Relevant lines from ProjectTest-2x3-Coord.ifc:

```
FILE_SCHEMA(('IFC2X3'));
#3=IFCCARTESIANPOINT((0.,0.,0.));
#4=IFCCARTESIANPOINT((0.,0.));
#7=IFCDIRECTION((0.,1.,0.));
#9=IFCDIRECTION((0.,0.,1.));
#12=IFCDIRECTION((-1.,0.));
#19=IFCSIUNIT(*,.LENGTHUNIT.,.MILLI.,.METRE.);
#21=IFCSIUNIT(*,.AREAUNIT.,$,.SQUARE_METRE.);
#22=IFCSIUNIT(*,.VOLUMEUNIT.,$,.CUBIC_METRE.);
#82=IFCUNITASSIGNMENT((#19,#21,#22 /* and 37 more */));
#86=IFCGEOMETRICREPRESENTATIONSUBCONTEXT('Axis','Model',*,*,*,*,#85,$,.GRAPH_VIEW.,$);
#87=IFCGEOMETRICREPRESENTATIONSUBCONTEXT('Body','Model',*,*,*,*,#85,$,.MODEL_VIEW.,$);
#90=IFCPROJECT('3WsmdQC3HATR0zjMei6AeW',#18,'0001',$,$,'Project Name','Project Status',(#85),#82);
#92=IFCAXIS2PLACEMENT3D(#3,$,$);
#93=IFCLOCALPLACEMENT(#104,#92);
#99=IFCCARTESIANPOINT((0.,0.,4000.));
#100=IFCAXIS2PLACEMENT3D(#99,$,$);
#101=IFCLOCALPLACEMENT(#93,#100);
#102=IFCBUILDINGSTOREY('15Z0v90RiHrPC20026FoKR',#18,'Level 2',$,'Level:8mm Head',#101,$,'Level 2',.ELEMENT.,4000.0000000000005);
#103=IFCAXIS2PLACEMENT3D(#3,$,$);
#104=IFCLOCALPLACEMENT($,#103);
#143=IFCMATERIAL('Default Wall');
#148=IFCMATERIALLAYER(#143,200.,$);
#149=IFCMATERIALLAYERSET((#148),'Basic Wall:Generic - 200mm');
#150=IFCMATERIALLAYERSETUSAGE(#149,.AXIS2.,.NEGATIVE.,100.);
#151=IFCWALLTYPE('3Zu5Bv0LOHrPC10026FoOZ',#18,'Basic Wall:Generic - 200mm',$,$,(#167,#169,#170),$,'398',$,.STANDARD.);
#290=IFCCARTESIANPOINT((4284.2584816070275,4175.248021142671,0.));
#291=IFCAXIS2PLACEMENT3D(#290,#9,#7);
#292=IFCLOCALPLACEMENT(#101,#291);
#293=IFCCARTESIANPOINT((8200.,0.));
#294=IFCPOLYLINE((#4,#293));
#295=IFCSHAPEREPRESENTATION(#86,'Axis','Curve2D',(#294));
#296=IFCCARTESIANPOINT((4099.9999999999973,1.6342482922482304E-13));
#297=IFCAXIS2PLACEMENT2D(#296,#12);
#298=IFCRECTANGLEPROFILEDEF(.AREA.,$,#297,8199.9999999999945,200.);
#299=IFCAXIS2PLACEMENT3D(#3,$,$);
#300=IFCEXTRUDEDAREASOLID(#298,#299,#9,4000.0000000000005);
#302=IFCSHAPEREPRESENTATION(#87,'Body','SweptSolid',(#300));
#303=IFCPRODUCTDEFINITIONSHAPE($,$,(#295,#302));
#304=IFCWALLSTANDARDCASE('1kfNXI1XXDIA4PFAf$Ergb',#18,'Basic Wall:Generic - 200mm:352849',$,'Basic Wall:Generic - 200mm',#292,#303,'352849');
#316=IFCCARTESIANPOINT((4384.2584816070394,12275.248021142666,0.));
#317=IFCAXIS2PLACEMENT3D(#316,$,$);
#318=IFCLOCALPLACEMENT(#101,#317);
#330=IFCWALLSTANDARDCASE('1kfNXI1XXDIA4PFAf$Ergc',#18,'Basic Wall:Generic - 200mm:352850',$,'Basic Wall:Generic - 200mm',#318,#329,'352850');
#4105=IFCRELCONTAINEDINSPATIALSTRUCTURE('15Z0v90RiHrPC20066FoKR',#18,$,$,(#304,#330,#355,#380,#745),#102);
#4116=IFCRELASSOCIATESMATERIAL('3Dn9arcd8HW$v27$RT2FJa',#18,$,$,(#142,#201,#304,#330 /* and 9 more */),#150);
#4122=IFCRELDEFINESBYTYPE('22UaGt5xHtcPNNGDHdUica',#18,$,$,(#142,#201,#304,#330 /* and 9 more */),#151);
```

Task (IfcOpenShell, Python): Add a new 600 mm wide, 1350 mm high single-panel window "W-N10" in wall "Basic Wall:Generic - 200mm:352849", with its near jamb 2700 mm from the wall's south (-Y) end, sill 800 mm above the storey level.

```python
import numpy as np
import ifcopenshell
import ifcopenshell.api.feature
import ifcopenshell.api.geometry
import ifcopenshell.api.root
import ifcopenshell.api.spatial
import ifcopenshell.api.type
import ifcopenshell.geom
import ifcopenshell.util.element
import ifcopenshell.util.placement
import ifcopenshell.util.representation
import ifcopenshell.util.shape
import ifcopenshell.util.unit

model = ifcopenshell.open("ProjectTest-2x3-Coord.ifc")
unit_scale = ifcopenshell.util.unit.calculate_unit_scale(model)
settings = ifcopenshell.geom.settings()


def volume(element):
    """Net volume in cubic metres, openings subtracted."""
    shape = ifcopenshell.geom.create_shape(settings, element)
    return ifcopenshell.util.shape.get_volume(shape.geometry)


wall = model.by_guid("1kfNXI1XXDIA4PFAf$Ergb")
storey = ifcopenshell.util.element.get_container(wall, ifc_class="IfcBuildingStorey")
context = ifcopenshell.util.representation.get_context(model, "Model", "Body", "MODEL_VIEW")
before = volume(wall)

width, height, from_end, sill = 0.6, 1.35, 2.7, 0.8  # metres

# The wall runs along its own X axis, and the end named is its -X end.
wall_shape = ifcopenshell.geom.create_shape(settings, wall)
x, y, z = ifcopenshell.util.shape.get_vertices(wall_shape.geometry).T
start = x.min() + from_end
face, thickness = float(y.min()), float(y.max() - y.min())
wall_matrix = ifcopenshell.util.placement.get_local_placement(wall.ObjectPlacement)
level = ifcopenshell.util.placement.get_local_placement(storey.ObjectPlacement)[2, 3]


def in_wall(x, y):
    """Placement at x, y metres in the wall's axes, at sill height."""
    matrix = wall_matrix.copy()
    matrix[:, 3] = wall_matrix @ np.array([x / unit_scale, y / unit_scale, 0.0, 1.0])
    matrix[2, 3] = level + sill / unit_scale
    return matrix


# Opening: a box that overshoots both wall faces by 50 mm.
opening = ifcopenshell.api.root.create_entity(model, ifc_class="IfcOpeningElement")
box = ifcopenshell.api.geometry.add_wall_representation(
    model, context=context, length=width, height=height, thickness=thickness + 0.1
)
ifcopenshell.api.geometry.assign_representation(model, product=opening, representation=box)
ifcopenshell.api.geometry.edit_object_placement(model, product=opening, matrix=in_wall(start, face - 0.05), is_si=False)
ifcopenshell.api.feature.add_feature(model, feature=opening, element=wall)

window = ifcopenshell.api.root.create_entity(model, ifc_class="IfcWindow", name="W-N10")
window.OverallWidth, window.OverallHeight = width / unit_scale, height / unit_scale
body = ifcopenshell.api.geometry.add_window_representation(
    model,
    context=context,
    overall_width=window.OverallWidth,
    overall_height=window.OverallHeight,
    partition_type="SINGLE_PANEL",
)
ifcopenshell.api.geometry.assign_representation(model, product=window, representation=body)
ifcopenshell.api.spatial.assign_container(model, products=[window], relating_structure=storey)
fills = ifcopenshell.api.feature.add_filling(model, opening=opening, element=window)
fills.OwnerHistory = window.OwnerHistory  # required in IFC2X3

# IFC2X3 keeps the operation on the window style.
style = ifcopenshell.api.root.create_entity(model, ifc_class="IfcWindowStyle", name="W-N10")
style.OperationType, style.ConstructionType = "SINGLE_PANEL", "NOTDEFINED"
style.ParameterTakesPrecedence = style.Sizeable = False
ifcopenshell.api.type.assign_type(model, related_objects=[window], relating_type=style)

# Centre the window in the wall's thickness.
ifcopenshell.api.geometry.edit_object_placement(model, product=window, matrix=in_wall(start, face), is_si=False)
window_shape = ifcopenshell.geom.create_shape(settings, window)
depth = ifcopenshell.util.shape.get_vertices(window_shape.geometry)[:, 1]
offset = face + thickness / 2 - (depth.min() + depth.max()) / 2
ifcopenshell.api.geometry.edit_object_placement(model, product=window, matrix=in_wall(start, offset), is_si=False)

after = volume(wall)

print(f"wall volume {before:.3f} -> {after:.3f} m3")

model.write("ProjectTest-2x3-Coord_edited.ifc")
```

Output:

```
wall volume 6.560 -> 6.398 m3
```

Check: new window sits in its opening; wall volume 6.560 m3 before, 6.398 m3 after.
